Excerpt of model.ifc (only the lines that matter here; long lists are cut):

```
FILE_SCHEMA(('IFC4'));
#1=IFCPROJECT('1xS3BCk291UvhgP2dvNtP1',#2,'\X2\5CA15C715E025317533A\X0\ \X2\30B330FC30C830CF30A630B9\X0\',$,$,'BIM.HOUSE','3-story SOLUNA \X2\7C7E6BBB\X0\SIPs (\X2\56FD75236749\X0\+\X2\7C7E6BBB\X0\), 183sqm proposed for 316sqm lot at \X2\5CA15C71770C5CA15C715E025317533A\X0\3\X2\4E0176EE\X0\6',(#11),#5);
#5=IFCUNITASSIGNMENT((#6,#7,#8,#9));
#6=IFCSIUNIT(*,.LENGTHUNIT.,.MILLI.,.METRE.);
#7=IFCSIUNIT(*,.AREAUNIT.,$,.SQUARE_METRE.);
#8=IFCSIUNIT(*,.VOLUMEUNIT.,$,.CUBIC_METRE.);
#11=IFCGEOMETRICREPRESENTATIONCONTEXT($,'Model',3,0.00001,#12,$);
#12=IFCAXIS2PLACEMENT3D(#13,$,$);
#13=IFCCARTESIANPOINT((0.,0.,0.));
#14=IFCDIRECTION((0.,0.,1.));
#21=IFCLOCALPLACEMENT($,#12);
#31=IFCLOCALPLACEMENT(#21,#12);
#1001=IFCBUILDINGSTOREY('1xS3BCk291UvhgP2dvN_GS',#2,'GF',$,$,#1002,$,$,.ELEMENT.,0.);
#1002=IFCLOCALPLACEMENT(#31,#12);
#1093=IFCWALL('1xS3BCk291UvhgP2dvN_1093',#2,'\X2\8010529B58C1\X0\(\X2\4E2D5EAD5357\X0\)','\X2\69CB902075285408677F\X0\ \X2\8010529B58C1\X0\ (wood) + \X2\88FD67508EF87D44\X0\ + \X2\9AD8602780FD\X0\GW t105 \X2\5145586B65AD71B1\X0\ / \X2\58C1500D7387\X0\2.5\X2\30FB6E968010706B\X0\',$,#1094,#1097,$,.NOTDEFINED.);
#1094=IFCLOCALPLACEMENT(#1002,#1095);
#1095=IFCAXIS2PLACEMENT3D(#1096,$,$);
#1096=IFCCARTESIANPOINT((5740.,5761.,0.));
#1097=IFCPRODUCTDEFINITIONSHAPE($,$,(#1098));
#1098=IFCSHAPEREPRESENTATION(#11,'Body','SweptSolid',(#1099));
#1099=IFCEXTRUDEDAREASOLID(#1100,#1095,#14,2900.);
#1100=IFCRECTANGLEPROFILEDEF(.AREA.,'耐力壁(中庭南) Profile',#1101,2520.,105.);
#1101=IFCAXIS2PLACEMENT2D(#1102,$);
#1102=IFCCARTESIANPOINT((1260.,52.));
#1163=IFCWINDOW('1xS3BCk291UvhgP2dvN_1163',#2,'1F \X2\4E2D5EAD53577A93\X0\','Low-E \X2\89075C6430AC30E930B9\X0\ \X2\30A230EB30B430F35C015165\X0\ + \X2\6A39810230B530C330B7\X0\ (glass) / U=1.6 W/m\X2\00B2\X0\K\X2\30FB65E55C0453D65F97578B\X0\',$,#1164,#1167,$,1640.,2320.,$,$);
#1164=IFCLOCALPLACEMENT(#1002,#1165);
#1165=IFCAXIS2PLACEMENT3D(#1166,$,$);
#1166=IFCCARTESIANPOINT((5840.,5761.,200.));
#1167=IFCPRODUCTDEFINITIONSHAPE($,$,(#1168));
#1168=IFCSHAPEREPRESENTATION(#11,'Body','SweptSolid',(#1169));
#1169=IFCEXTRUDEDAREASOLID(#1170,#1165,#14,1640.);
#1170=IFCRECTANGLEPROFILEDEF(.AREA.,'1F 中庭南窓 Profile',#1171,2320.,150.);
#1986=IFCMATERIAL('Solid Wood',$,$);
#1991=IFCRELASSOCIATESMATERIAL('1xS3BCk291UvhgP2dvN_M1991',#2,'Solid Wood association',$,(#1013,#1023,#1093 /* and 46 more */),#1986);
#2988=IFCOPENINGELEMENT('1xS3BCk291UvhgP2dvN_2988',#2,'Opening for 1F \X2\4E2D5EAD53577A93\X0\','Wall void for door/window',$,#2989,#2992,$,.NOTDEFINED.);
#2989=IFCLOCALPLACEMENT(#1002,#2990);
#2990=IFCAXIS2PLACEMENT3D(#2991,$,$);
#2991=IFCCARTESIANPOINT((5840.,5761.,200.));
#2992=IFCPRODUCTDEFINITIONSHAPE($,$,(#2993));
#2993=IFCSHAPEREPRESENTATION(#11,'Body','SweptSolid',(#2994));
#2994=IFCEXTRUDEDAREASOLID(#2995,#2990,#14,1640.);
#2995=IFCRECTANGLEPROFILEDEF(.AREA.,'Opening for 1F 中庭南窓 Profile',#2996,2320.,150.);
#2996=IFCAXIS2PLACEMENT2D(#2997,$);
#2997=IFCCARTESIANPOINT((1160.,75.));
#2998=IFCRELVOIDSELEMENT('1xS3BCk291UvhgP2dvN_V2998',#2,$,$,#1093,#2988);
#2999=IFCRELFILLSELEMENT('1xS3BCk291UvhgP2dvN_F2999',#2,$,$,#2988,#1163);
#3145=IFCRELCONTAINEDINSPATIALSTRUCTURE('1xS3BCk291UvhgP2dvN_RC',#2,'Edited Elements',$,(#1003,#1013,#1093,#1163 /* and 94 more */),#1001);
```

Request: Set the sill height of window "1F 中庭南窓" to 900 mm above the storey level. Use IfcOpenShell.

```python
import numpy as np
import ifcopenshell
import ifcopenshell.api.geometry
import ifcopenshell.geom
import ifcopenshell.util.element
import ifcopenshell.util.placement
import ifcopenshell.util.shape
import ifcopenshell.util.unit

model = ifcopenshell.open("model.ifc")
unit_scale = ifcopenshell.util.unit.calculate_unit_scale(model)

window = model.by_guid("1xS3BCk291UvhgP2dvN_1163")
opening = window.FillsVoids[0].RelatingOpeningElement
storey = ifcopenshell.util.element.get_container(window, ifc_class="IfcBuildingStorey")
level = ifcopenshell.util.placement.get_local_placement(storey.ObjectPlacement)[2, 3]

# The opening's origin need not be at the sill, so measure its lowest point.
shape = ifcopenshell.geom.create_shape(ifcopenshell.geom.settings(), opening)
bottom = ifcopenshell.util.shape.get_shape_bottom_elevation(shape, shape.geometry) / unit_scale
dz = level + 900.0 - bottom

shift = np.array([0.0, 0.0, dz])
# The window is not placed relative to its opening, so move both.
for product in (opening, window):
    matrix = ifcopenshell.util.placement.get_local_placement(product.ObjectPlacement)
    matrix[:3, 3] += shift
    ifcopenshell.api.geometry.edit_object_placement(model, product=product, matrix=matrix, is_si=False)

print(f"moved by {dz * unit_scale:+.3f} m")

model.write("model_updated.ifc")
```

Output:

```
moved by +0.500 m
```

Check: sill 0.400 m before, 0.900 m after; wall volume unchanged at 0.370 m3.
